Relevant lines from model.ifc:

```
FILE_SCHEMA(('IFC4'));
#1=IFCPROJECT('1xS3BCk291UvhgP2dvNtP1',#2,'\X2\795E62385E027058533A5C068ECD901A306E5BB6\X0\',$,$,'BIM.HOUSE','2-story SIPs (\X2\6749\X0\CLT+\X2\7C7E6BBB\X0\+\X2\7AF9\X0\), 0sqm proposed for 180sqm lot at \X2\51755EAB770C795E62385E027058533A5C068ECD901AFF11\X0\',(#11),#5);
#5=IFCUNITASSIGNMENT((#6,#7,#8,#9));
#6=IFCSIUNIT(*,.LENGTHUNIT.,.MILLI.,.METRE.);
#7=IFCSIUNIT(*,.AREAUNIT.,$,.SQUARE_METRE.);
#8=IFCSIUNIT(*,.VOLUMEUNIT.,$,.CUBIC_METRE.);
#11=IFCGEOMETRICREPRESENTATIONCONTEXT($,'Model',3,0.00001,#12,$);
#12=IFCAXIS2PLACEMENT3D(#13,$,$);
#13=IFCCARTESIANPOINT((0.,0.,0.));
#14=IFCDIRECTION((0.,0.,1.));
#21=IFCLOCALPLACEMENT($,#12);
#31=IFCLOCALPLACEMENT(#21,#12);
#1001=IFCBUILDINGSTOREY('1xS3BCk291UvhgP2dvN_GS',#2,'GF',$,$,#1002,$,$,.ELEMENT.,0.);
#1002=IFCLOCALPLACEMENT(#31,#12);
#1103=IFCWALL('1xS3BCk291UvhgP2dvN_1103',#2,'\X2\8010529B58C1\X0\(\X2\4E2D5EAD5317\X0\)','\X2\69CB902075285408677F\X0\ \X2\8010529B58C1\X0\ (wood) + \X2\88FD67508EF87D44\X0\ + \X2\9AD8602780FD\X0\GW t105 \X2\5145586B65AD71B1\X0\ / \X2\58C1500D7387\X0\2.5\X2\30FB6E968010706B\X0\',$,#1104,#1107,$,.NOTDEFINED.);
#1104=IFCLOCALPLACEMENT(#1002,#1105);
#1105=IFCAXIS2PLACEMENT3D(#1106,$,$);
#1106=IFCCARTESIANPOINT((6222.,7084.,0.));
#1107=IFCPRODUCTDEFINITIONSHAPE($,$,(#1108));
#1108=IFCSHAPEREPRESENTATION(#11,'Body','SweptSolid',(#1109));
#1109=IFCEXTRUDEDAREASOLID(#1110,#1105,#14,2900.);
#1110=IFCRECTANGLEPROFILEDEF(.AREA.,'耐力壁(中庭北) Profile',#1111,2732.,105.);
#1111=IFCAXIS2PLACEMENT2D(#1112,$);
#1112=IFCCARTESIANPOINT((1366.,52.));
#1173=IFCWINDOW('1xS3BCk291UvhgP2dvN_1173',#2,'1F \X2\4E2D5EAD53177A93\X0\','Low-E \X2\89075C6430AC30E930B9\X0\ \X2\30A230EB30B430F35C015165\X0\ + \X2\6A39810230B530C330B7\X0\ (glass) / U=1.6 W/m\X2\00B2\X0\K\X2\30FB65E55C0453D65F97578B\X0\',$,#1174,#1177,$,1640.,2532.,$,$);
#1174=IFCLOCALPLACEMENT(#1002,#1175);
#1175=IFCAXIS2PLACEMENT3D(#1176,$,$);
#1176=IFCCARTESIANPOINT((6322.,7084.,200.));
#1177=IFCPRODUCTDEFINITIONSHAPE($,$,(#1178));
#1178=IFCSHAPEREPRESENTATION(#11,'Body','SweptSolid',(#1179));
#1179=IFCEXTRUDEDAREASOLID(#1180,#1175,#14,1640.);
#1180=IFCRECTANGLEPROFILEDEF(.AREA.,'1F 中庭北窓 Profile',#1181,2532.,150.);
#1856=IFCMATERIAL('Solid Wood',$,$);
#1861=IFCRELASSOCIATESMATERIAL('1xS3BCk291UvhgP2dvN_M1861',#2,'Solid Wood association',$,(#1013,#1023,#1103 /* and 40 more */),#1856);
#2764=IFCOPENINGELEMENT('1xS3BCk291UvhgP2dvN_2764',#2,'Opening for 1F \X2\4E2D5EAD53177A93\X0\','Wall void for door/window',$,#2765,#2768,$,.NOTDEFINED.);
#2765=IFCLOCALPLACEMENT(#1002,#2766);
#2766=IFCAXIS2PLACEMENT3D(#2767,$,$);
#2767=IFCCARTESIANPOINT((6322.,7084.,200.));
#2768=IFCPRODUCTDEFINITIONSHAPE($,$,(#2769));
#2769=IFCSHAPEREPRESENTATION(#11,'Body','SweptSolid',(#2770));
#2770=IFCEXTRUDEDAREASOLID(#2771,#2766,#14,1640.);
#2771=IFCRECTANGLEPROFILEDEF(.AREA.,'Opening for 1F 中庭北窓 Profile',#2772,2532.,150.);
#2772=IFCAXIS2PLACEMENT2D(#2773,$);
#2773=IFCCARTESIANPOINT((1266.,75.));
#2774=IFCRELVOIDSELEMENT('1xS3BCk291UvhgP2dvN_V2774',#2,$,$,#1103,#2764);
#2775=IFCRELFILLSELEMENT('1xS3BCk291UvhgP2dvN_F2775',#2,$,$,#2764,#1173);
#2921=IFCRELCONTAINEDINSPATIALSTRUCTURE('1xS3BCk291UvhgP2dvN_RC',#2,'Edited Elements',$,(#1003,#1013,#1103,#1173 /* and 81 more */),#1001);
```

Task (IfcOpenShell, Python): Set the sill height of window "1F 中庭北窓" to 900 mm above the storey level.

```python
import numpy as np
import ifcopenshell
import ifcopenshell.api.geometry
import ifcopenshell.geom
import ifcopenshell.util.element
import ifcopenshell.util.placement
import ifcopenshell.util.shape
import ifcopenshell.util.unit

model = ifcopenshell.open("model.ifc")
unit_scale = ifcopenshell.util.unit.calculate_unit_scale(model)

window = model.by_guid("1xS3BCk291UvhgP2dvN_1173")
opening = window.FillsVoids[0].RelatingOpeningElement
storey = ifcopenshell.util.element.get_container(window, ifc_class="IfcBuildingStorey")
level = ifcopenshell.util.placement.get_local_placement(storey.ObjectPlacement)[2, 3]

# The opening's origin need not be at the sill, so measure its lowest point.
shape = ifcopenshell.geom.create_shape(ifcopenshell.geom.settings(), opening)
bottom = ifcopenshell.util.shape.get_shape_bottom_elevation(shape, shape.geometry) / unit_scale
dz = level + 900.0 - bottom

shift = np.array([0.0, 0.0, dz])
# The window is not placed relative to its opening, so move both.
for product in (opening, window):
    matrix = ifcopenshell.util.placement.get_local_placement(product.ObjectPlacement)
    matrix[:3, 3] += shift
    ifcopenshell.api.geometry.edit_object_placement(model, product=product, matrix=matrix, is_si=False)

print(f"moved by {dz * unit_scale:+.3f} m")

model.write("model-out.ifc")
```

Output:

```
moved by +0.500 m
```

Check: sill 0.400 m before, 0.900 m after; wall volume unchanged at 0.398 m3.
